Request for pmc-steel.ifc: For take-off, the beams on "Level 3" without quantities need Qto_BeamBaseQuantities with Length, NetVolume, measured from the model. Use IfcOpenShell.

First a look at what the model holds.

```python
import ifcopenshell
import ifcopenshell.util.element
import ifcopenshell.util.unit

model = ifcopenshell.open("pmc-steel.ifc")
print(model.schema)
for unit_type in ("LENGTHUNIT", "AREAUNIT", "VOLUMEUNIT"):
    print(unit_type, ifcopenshell.util.unit.calculate_unit_scale(model, unit_type))
storey = next(s for s in model.by_type("IfcBuildingStorey") if s.Name == "Level 3")
beams = [e for e in ifcopenshell.util.element.get_decomposition(storey) if e.is_a("IfcBeam")]
for e in sorted(beams, key=lambda e: e.id()):
    print(e.id(), e.is_a(), e.Name, list(ifcopenshell.util.element.get_psets(e, qtos_only=True)), sep=" | ")
```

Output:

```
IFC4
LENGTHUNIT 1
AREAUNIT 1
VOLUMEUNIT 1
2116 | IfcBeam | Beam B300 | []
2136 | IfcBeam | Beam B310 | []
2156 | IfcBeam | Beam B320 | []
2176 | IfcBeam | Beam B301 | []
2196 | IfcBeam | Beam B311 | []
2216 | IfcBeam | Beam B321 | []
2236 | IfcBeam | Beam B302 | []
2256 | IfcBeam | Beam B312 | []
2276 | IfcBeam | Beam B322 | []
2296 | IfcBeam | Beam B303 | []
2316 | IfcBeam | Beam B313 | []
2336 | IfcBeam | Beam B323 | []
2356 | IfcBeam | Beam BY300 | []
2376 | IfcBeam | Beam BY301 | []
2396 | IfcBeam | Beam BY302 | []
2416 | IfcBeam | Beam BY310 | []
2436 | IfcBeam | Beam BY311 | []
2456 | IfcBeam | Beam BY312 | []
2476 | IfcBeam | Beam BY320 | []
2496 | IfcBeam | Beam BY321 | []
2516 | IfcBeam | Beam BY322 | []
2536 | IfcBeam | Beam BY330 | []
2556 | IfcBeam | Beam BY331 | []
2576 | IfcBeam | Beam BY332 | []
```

```python
import ifcopenshell
import ifcopenshell.api.pset
import ifcopenshell.geom
import ifcopenshell.util.element
import ifcopenshell.util.shape
import ifcopenshell.util.unit

model = ifcopenshell.open("pmc-steel.ifc")
unit_scale = ifcopenshell.util.unit.calculate_unit_scale(model)
volume_scale = ifcopenshell.util.unit.calculate_unit_scale(model, "VOLUMEUNIT")
settings = ifcopenshell.geom.settings()

storey = next(s for s in model.by_type("IfcBuildingStorey") if s.Name == "Level 3")
beams = [e for e in ifcopenshell.util.element.get_decomposition(storey) if e.is_a("IfcBeam")]

for e in sorted(beams, key=lambda e: e.id()):
    if ifcopenshell.util.element.get_psets(e, qtos_only=True, should_inherit=False):
        continue
    # Geometry comes back in metres, in the element's own axes.
    shape = ifcopenshell.geom.create_shape(settings, e)
    values = {
        "Length": ifcopenshell.util.shape.get_max_xyz(shape.geometry) / unit_scale,
        "NetVolume": ifcopenshell.util.shape.get_volume(shape.geometry) / volume_scale,
    }
    qto = ifcopenshell.api.pset.add_qto(model, product=e, name="Qto_BeamBaseQuantities")
    ifcopenshell.api.pset.edit_qto(model, qto=qto, properties=values)
    print(e.id(), {k: round(v, 3) for k, v in values.items()})

model.write("pmc-steel-out.ifc")
```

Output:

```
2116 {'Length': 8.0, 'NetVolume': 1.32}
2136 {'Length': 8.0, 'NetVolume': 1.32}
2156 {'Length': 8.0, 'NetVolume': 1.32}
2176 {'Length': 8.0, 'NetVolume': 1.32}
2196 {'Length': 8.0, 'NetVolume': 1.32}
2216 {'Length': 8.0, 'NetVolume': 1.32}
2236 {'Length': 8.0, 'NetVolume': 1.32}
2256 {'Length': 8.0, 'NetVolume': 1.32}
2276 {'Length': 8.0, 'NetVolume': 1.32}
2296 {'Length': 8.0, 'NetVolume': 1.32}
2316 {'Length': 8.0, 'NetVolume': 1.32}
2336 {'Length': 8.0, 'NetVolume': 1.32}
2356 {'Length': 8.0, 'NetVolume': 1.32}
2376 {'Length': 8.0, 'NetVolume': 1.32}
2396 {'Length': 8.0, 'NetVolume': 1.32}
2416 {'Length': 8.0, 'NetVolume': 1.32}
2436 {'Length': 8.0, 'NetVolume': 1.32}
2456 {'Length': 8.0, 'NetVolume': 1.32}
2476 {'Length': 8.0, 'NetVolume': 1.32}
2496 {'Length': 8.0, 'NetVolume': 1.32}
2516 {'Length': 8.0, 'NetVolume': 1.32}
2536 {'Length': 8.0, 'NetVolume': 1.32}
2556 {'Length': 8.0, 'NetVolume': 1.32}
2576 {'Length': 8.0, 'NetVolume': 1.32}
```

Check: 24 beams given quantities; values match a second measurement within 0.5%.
